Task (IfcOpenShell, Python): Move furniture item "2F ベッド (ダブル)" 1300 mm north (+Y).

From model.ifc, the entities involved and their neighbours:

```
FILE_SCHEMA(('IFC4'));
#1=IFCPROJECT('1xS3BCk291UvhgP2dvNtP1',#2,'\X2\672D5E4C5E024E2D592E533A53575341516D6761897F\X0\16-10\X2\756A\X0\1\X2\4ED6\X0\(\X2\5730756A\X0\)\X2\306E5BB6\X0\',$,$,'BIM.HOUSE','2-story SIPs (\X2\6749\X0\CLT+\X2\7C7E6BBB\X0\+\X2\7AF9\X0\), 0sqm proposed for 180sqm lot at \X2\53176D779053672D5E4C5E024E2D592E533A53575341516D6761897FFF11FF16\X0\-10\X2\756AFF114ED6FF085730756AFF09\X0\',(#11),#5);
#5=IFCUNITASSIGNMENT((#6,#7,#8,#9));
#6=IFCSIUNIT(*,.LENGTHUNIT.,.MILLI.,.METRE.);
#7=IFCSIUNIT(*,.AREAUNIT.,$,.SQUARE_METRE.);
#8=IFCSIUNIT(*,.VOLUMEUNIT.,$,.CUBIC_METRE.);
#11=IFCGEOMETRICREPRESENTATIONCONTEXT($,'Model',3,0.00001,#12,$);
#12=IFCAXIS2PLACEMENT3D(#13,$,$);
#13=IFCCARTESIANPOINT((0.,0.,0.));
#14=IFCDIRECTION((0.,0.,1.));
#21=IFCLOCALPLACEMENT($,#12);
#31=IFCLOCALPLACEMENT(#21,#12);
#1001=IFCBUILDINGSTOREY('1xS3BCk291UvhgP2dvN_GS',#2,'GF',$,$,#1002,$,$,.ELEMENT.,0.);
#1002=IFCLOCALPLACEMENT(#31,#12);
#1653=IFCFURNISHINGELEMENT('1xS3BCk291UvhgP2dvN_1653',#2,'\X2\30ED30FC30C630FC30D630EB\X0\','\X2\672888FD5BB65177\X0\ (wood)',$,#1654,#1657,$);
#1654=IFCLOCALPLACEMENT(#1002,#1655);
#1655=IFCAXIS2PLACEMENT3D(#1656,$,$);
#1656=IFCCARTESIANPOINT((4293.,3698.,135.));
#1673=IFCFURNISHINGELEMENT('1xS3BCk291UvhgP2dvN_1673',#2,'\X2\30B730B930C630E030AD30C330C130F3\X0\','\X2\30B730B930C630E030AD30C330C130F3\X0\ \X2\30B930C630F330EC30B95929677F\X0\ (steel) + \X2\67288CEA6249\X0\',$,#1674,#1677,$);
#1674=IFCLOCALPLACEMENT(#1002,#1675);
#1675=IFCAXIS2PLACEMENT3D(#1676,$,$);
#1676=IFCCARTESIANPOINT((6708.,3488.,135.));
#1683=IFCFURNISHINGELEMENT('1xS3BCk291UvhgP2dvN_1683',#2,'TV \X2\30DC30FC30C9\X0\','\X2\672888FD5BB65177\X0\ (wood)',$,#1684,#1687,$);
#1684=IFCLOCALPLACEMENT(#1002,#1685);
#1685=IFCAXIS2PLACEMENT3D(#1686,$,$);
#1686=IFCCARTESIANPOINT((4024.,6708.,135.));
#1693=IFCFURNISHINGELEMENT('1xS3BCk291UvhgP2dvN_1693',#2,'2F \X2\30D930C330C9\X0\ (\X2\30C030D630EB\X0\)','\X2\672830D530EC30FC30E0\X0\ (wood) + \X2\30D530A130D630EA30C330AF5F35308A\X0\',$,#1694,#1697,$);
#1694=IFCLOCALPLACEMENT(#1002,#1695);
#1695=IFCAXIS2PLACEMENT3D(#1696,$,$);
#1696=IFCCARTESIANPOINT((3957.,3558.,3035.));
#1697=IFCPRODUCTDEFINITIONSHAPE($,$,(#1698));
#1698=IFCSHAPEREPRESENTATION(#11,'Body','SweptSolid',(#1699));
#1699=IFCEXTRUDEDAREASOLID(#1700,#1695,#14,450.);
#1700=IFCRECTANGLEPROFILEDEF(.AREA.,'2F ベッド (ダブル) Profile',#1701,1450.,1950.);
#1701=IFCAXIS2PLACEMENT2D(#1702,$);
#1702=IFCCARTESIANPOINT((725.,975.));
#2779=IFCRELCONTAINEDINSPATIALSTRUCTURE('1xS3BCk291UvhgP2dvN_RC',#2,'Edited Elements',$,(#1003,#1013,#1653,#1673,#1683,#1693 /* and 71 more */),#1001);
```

```python
import ifcopenshell
import ifcopenshell.api.geometry
import ifcopenshell.util.placement

model = ifcopenshell.open("model.ifc")

item = model.by_guid("1xS3BCk291UvhgP2dvN_1693")
matrix = ifcopenshell.util.placement.get_local_placement(item.ObjectPlacement)
matrix[1, 3] += 1300.0
ifcopenshell.api.geometry.edit_object_placement(model, product=item, matrix=matrix, is_si=False)

print(ifcopenshell.util.placement.get_local_placement(item.ObjectPlacement).round(3) + 0.0)

model.write("model-out.ifc")
```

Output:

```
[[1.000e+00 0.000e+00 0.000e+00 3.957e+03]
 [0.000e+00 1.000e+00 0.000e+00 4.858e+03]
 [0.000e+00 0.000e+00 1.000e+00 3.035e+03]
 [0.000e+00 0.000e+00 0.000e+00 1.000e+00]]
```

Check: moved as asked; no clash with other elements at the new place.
